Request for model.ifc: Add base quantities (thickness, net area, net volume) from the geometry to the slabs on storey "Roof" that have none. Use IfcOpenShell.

First a look at what the model holds.

```python
import ifcopenshell
import ifcopenshell.util.element
import ifcopenshell.util.unit

model = ifcopenshell.open("model.ifc")
print(model.schema)
for unit_type in ("LENGTHUNIT", "AREAUNIT", "VOLUMEUNIT"):
    print(unit_type, ifcopenshell.util.unit.calculate_unit_scale(model, unit_type))
storey = next(s for s in model.by_type("IfcBuildingStorey") if s.Name == "Roof")
slabs = [e for e in ifcopenshell.util.element.get_decomposition(storey) if e.is_a("IfcSlab")]
for e in sorted(slabs, key=lambda e: e.id()):
    print(e.id(), e.is_a(), e.Name, list(ifcopenshell.util.element.get_psets(e, qtos_only=True)), sep=" | ")
```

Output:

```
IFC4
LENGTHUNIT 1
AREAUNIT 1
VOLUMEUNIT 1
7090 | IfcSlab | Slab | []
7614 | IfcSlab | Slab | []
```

```python
import ifcopenshell
import ifcopenshell.api.pset
import ifcopenshell.geom
import ifcopenshell.util.element
import ifcopenshell.util.shape
import ifcopenshell.util.unit

model = ifcopenshell.open("model.ifc")
unit_scale = ifcopenshell.util.unit.calculate_unit_scale(model)
area_scale = ifcopenshell.util.unit.calculate_unit_scale(model, "AREAUNIT")
volume_scale = ifcopenshell.util.unit.calculate_unit_scale(model, "VOLUMEUNIT")
settings = ifcopenshell.geom.settings()

storey = next(s for s in model.by_type("IfcBuildingStorey") if s.Name == "Roof")
slabs = [e for e in ifcopenshell.util.element.get_decomposition(storey) if e.is_a("IfcSlab")]

for e in sorted(slabs, key=lambda e: e.id()):
    if ifcopenshell.util.element.get_psets(e, qtos_only=True, should_inherit=False):
        continue
    # Geometry comes back in metres, in the element's own axes.
    shape = ifcopenshell.geom.create_shape(settings, e)
    values = {
        "Width": ifcopenshell.util.shape.get_z(shape.geometry) / unit_scale,
        "NetArea": ifcopenshell.util.shape.get_footprint_area(shape.geometry) / area_scale,
        "NetVolume": ifcopenshell.util.shape.get_volume(shape.geometry) / volume_scale,
    }
    qto = ifcopenshell.api.pset.add_qto(model, product=e, name="Qto_SlabBaseQuantities")
    ifcopenshell.api.pset.edit_qto(model, qto=qto, properties=values)
    print(e.id(), {k: round(v, 3) for k, v in values.items()})

model.write("model-out.ifc")
```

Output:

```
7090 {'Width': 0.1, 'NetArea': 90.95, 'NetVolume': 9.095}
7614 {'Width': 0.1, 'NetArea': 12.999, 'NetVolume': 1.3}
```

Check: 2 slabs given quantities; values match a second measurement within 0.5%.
